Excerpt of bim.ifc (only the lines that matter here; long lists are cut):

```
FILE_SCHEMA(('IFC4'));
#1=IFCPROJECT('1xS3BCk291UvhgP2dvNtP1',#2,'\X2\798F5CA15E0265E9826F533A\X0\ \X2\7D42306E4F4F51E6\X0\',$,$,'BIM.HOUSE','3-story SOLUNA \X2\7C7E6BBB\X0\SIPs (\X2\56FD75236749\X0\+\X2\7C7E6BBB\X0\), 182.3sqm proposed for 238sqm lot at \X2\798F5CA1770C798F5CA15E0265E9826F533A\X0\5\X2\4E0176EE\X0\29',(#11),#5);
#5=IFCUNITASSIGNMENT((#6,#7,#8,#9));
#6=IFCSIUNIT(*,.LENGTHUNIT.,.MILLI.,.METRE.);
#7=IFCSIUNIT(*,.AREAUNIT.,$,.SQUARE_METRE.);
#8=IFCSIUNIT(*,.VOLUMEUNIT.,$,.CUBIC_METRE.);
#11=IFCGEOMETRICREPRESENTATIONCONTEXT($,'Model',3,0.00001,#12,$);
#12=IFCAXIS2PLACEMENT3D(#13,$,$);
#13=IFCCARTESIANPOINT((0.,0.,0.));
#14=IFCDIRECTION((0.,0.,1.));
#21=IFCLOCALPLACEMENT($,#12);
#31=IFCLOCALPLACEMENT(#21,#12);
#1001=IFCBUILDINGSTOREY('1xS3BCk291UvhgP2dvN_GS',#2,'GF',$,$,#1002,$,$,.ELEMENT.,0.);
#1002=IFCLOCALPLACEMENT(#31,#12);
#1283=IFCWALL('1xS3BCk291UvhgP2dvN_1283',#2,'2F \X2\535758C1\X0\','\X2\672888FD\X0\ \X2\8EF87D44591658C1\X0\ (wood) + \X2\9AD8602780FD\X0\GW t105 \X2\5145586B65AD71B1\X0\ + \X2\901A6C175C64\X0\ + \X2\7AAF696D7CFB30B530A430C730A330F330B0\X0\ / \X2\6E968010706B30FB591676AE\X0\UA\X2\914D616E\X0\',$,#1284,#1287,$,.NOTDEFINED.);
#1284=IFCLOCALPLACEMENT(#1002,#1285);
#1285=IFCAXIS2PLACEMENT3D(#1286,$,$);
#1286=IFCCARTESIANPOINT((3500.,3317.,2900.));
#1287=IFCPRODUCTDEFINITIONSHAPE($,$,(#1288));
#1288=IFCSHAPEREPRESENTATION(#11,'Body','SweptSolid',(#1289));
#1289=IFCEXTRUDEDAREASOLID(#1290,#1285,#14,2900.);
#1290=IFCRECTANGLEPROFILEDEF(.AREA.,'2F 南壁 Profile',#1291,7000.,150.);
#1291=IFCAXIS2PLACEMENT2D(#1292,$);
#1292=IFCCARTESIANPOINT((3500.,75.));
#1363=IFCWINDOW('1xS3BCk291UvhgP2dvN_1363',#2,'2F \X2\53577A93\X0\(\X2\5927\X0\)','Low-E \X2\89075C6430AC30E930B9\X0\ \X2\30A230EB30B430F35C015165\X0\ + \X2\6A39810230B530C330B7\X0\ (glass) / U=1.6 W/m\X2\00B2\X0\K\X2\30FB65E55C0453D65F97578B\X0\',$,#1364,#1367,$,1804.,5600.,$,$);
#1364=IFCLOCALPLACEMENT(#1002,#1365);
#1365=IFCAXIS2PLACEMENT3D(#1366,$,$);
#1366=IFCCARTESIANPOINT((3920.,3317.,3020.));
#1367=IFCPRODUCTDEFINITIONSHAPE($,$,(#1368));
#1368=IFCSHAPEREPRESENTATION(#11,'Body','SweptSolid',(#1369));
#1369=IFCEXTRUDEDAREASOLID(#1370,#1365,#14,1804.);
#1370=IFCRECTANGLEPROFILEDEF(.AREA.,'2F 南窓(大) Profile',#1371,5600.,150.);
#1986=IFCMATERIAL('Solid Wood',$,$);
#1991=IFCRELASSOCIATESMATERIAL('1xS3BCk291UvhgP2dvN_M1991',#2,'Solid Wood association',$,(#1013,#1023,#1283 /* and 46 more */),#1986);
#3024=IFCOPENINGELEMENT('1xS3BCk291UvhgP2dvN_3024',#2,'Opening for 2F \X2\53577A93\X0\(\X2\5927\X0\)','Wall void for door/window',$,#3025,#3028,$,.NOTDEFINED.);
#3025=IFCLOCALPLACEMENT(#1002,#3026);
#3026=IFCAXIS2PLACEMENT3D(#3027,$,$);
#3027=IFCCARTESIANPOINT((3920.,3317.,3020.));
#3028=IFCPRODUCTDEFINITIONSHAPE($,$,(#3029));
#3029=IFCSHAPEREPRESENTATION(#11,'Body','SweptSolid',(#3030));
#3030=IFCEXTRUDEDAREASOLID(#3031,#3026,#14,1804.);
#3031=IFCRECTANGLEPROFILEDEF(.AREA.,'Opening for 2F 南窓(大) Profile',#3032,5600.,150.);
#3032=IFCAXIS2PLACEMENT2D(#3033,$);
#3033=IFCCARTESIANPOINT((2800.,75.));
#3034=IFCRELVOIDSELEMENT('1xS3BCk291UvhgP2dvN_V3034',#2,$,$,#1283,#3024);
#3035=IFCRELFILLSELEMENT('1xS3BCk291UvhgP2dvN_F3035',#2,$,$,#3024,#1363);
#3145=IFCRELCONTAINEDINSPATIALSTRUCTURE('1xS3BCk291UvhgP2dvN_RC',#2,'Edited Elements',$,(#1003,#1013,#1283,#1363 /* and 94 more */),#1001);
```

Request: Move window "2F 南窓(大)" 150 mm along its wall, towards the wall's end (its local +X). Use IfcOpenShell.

```python
import ifcopenshell
import ifcopenshell.api.geometry
import ifcopenshell.util.placement

model = ifcopenshell.open("bim.ifc")

window = model.by_guid("1xS3BCk291UvhgP2dvN_1363")
opening = window.FillsVoids[0].RelatingOpeningElement
wall = opening.VoidsElements[0].RelatingBuildingElement

wall_matrix = ifcopenshell.util.placement.get_local_placement(wall.ObjectPlacement)
shift = wall_matrix[:3, 0] * 150.0
before = ifcopenshell.util.placement.get_local_placement(window.ObjectPlacement)[:3, 3].copy()

# The window is not placed relative to its opening, so move both.
for product in (opening, window):
    matrix = ifcopenshell.util.placement.get_local_placement(product.ObjectPlacement)
    matrix[:3, 3] += shift
    ifcopenshell.api.geometry.edit_object_placement(model, product=product, matrix=matrix, is_si=False)

after = ifcopenshell.util.placement.get_local_placement(window.ObjectPlacement)[:3, 3]
print("window moved by", (after - before).round(3) + 0.0)

model.write("bim_updated.ifc")
```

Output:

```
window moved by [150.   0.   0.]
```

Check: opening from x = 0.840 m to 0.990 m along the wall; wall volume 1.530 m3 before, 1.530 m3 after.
